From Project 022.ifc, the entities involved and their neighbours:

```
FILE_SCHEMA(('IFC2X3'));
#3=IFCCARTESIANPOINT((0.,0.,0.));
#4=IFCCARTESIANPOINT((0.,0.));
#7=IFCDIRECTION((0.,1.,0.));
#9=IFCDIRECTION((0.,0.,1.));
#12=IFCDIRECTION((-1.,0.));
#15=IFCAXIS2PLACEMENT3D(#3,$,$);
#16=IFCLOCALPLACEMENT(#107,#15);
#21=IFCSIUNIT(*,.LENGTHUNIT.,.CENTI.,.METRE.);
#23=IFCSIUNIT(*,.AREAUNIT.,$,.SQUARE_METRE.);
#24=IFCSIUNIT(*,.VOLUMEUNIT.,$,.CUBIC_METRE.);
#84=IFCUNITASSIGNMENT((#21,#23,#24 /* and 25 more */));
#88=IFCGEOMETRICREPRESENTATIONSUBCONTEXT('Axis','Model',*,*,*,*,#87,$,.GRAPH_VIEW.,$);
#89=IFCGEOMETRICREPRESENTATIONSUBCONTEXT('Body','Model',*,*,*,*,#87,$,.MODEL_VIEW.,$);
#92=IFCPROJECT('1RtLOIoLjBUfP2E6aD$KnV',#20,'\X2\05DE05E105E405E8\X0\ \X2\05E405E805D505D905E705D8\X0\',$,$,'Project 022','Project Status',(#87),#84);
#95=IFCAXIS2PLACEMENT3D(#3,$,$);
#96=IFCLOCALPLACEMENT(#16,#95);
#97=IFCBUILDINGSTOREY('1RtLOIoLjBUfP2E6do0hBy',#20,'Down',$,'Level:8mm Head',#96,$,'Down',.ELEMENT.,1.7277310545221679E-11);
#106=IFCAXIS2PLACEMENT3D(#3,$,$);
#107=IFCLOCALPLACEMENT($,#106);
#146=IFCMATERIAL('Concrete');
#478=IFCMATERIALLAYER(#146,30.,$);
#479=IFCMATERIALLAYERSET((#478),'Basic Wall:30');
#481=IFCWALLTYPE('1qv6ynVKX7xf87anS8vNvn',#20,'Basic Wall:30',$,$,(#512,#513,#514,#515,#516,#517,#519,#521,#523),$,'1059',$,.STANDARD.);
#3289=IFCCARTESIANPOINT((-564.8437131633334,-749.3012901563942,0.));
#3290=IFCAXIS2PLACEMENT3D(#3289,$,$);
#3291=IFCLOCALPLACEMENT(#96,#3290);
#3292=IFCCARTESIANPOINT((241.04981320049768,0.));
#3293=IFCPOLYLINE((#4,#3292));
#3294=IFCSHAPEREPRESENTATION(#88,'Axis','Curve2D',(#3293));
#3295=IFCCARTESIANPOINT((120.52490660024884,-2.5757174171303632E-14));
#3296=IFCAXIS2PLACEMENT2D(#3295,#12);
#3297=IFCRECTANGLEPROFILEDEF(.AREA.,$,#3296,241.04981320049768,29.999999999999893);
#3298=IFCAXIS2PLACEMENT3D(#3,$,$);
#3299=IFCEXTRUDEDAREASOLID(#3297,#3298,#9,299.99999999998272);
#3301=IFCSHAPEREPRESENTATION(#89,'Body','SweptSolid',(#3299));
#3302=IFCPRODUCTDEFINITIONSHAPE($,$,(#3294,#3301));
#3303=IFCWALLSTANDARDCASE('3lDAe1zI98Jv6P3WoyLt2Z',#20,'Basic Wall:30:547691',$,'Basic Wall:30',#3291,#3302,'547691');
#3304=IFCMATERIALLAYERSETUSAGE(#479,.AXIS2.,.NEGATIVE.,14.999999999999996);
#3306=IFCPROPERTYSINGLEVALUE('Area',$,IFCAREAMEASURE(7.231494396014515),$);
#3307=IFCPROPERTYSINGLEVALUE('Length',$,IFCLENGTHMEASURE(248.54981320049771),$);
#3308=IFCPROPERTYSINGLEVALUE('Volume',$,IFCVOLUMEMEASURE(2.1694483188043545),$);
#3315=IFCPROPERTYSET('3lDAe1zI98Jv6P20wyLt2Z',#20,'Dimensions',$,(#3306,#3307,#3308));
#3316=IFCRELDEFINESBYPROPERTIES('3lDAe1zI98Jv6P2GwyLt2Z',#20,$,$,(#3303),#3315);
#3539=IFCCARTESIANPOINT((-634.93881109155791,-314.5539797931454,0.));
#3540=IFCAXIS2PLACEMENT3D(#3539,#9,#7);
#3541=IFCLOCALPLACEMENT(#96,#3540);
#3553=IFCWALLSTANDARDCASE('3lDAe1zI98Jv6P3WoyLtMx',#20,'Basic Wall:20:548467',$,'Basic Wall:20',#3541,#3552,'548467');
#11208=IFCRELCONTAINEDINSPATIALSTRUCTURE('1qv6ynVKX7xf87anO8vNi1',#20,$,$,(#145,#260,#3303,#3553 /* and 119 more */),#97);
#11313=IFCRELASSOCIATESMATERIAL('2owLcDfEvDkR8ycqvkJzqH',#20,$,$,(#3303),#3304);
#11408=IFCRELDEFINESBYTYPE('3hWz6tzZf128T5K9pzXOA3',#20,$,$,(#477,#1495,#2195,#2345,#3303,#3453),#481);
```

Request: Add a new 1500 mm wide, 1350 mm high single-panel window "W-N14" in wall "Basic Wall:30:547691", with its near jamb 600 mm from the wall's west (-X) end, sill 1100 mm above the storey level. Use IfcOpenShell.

```python
import numpy as np
import ifcopenshell
import ifcopenshell.api.feature
import ifcopenshell.api.geometry
import ifcopenshell.api.pset
import ifcopenshell.api.root
import ifcopenshell.api.spatial
import ifcopenshell.api.type
import ifcopenshell.geom
import ifcopenshell.util.element
import ifcopenshell.util.placement
import ifcopenshell.util.representation
import ifcopenshell.util.shape
import ifcopenshell.util.unit

model = ifcopenshell.open("Project 022.ifc")
unit_scale = ifcopenshell.util.unit.calculate_unit_scale(model)
area_scale = ifcopenshell.util.unit.calculate_unit_scale(model, "AREAUNIT")
volume_scale = ifcopenshell.util.unit.calculate_unit_scale(model, "VOLUMEUNIT")
settings = ifcopenshell.geom.settings()


def volume(element):
    """Net volume in cubic metres, openings subtracted."""
    shape = ifcopenshell.geom.create_shape(settings, element)
    return ifcopenshell.util.shape.get_volume(shape.geometry)


wall = model.by_guid("3lDAe1zI98Jv6P3WoyLt2Z")
storey = ifcopenshell.util.element.get_container(wall, ifc_class="IfcBuildingStorey")
context = ifcopenshell.util.representation.get_context(model, "Model", "Body", "MODEL_VIEW")
before = volume(wall)

width, height, from_end, sill = 1.5, 1.35, 0.6, 1.1  # metres

# The wall runs along its own X axis, and the end named is its -X end.
wall_shape = ifcopenshell.geom.create_shape(settings, wall)
x, y, z = ifcopenshell.util.shape.get_vertices(wall_shape.geometry).T
start = x.min() + from_end
face, thickness = float(y.min()), float(y.max() - y.min())
wall_matrix = ifcopenshell.util.placement.get_local_placement(wall.ObjectPlacement)
level = ifcopenshell.util.placement.get_local_placement(storey.ObjectPlacement)[2, 3]


def in_wall(x, y):
    """Placement at x, y metres in the wall's axes, at sill height."""
    matrix = wall_matrix.copy()
    matrix[:, 3] = wall_matrix @ np.array([x / unit_scale, y / unit_scale, 0.0, 1.0])
    matrix[2, 3] = level + sill / unit_scale
    return matrix


# Opening: a box that overshoots both wall faces by 50 mm.
opening = ifcopenshell.api.root.create_entity(model, ifc_class="IfcOpeningElement")
box = ifcopenshell.api.geometry.add_wall_representation(
    model, context=context, length=width, height=height, thickness=thickness + 0.1
)
ifcopenshell.api.geometry.assign_representation(model, product=opening, representation=box)
ifcopenshell.api.geometry.edit_object_placement(model, product=opening, matrix=in_wall(start, face - 0.05), is_si=False)
ifcopenshell.api.feature.add_feature(model, feature=opening, element=wall)

window = ifcopenshell.api.root.create_entity(model, ifc_class="IfcWindow", name="W-N14")
window.OverallWidth, window.OverallHeight = width / unit_scale, height / unit_scale
body = ifcopenshell.api.geometry.add_window_representation(
    model,
    context=context,
    overall_width=window.OverallWidth,
    overall_height=window.OverallHeight,
    partition_type="SINGLE_PANEL",
)
ifcopenshell.api.geometry.assign_representation(model, product=window, representation=body)
ifcopenshell.api.spatial.assign_container(model, products=[window], relating_structure=storey)
fills = ifcopenshell.api.feature.add_filling(model, opening=opening, element=window)
fills.OwnerHistory = window.OwnerHistory  # required in IFC2X3

# IFC2X3 keeps the operation on the window style.
style = ifcopenshell.api.root.create_entity(model, ifc_class="IfcWindowStyle", name="W-N14")
style.OperationType, style.ConstructionType = "SINGLE_PANEL", "NOTDEFINED"
style.ParameterTakesPrecedence = style.Sizeable = False
ifcopenshell.api.type.assign_type(model, related_objects=[window], relating_type=style)

# Centre the window in the wall's thickness.
ifcopenshell.api.geometry.edit_object_placement(model, product=window, matrix=in_wall(start, face), is_si=False)
window_shape = ifcopenshell.geom.create_shape(settings, window)
depth = ifcopenshell.util.shape.get_vertices(window_shape.geometry)[:, 1]
offset = face + thickness / 2 - (depth.min() + depth.max()) / 2
ifcopenshell.api.geometry.edit_object_placement(model, product=window, matrix=in_wall(start, offset), is_si=False)

after = volume(wall)

# Update the wall's stored quantities.
pset = model.by_id(ifcopenshell.util.element.get_pset(wall, "Dimensions", should_inherit=False)["id"])
ifcopenshell.api.pset.edit_pset(model, pset=pset, properties={
    "Area": model.create_entity("IfcAreaMeasure", after / thickness / area_scale),
    "Volume": model.create_entity("IfcVolumeMeasure", after / volume_scale),
})

print(f"wall volume {before:.3f} -> {after:.3f} m3")

model.write("Project 022_v2.ifc")
```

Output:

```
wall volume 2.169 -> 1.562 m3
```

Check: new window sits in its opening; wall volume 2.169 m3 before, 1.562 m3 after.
